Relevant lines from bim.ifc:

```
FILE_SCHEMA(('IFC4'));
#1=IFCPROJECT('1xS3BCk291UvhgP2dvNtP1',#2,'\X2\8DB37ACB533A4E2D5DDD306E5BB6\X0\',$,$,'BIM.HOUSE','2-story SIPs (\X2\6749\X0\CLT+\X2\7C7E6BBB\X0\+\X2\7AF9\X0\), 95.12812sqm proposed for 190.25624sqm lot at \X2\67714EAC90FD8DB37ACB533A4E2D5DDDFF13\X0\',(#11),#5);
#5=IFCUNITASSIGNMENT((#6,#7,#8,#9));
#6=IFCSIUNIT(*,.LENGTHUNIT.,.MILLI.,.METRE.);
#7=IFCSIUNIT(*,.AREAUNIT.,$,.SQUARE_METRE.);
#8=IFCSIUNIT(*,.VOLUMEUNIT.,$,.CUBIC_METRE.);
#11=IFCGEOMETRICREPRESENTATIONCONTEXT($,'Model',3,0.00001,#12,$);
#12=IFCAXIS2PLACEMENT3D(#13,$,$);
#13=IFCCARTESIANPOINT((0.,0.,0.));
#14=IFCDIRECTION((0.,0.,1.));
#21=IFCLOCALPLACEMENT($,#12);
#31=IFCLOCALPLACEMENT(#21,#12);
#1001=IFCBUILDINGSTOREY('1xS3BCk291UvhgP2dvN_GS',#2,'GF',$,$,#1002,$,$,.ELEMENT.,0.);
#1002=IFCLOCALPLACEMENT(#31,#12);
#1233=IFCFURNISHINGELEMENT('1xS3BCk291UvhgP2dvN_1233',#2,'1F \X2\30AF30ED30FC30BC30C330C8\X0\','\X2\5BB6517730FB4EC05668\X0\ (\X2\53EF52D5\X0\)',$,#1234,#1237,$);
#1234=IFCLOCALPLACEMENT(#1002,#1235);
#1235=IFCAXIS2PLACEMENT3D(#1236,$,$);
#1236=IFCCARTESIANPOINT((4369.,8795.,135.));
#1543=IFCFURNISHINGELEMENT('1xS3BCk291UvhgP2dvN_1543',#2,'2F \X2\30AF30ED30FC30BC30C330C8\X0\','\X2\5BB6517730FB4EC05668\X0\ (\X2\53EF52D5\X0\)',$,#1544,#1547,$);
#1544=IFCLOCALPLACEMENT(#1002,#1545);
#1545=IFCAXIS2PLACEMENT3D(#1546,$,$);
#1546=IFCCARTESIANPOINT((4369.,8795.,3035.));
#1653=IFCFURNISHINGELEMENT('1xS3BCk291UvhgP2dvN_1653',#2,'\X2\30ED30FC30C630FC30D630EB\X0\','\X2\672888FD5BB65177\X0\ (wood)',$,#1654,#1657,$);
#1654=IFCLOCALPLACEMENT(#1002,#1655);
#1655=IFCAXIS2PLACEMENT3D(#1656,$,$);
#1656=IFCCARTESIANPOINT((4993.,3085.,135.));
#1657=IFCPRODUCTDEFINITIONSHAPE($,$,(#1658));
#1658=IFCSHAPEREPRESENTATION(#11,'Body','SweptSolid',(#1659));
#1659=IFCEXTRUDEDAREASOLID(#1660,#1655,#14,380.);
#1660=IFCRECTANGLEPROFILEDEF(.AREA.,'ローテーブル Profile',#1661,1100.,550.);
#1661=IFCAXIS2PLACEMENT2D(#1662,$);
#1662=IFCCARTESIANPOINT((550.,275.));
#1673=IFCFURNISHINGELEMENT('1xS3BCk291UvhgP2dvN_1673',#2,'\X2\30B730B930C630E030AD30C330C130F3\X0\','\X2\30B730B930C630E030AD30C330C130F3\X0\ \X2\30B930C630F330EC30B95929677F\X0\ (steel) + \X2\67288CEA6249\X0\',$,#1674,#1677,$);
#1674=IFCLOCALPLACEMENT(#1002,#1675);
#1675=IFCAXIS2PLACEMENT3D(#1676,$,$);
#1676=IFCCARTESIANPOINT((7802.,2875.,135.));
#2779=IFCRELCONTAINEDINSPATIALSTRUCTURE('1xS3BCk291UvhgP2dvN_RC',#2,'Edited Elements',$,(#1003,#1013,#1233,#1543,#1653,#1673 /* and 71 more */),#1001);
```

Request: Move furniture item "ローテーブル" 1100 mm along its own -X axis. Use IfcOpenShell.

```python
import ifcopenshell
import ifcopenshell.api.geometry
import ifcopenshell.util.placement

model = ifcopenshell.open("bim.ifc")

item = model.by_guid("1xS3BCk291UvhgP2dvN_1653")
matrix = ifcopenshell.util.placement.get_local_placement(item.ObjectPlacement)
matrix[:3, 3] -= matrix[:3, 0] * 1100.0
ifcopenshell.api.geometry.edit_object_placement(model, product=item, matrix=matrix, is_si=False)

print(ifcopenshell.util.placement.get_local_placement(item.ObjectPlacement).round(3) + 0.0)

model.write("bim_updated.ifc")
```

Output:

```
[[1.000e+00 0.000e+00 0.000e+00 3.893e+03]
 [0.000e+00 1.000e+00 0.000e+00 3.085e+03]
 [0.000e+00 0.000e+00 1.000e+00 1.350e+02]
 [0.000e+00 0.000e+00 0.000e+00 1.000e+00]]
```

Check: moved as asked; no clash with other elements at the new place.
